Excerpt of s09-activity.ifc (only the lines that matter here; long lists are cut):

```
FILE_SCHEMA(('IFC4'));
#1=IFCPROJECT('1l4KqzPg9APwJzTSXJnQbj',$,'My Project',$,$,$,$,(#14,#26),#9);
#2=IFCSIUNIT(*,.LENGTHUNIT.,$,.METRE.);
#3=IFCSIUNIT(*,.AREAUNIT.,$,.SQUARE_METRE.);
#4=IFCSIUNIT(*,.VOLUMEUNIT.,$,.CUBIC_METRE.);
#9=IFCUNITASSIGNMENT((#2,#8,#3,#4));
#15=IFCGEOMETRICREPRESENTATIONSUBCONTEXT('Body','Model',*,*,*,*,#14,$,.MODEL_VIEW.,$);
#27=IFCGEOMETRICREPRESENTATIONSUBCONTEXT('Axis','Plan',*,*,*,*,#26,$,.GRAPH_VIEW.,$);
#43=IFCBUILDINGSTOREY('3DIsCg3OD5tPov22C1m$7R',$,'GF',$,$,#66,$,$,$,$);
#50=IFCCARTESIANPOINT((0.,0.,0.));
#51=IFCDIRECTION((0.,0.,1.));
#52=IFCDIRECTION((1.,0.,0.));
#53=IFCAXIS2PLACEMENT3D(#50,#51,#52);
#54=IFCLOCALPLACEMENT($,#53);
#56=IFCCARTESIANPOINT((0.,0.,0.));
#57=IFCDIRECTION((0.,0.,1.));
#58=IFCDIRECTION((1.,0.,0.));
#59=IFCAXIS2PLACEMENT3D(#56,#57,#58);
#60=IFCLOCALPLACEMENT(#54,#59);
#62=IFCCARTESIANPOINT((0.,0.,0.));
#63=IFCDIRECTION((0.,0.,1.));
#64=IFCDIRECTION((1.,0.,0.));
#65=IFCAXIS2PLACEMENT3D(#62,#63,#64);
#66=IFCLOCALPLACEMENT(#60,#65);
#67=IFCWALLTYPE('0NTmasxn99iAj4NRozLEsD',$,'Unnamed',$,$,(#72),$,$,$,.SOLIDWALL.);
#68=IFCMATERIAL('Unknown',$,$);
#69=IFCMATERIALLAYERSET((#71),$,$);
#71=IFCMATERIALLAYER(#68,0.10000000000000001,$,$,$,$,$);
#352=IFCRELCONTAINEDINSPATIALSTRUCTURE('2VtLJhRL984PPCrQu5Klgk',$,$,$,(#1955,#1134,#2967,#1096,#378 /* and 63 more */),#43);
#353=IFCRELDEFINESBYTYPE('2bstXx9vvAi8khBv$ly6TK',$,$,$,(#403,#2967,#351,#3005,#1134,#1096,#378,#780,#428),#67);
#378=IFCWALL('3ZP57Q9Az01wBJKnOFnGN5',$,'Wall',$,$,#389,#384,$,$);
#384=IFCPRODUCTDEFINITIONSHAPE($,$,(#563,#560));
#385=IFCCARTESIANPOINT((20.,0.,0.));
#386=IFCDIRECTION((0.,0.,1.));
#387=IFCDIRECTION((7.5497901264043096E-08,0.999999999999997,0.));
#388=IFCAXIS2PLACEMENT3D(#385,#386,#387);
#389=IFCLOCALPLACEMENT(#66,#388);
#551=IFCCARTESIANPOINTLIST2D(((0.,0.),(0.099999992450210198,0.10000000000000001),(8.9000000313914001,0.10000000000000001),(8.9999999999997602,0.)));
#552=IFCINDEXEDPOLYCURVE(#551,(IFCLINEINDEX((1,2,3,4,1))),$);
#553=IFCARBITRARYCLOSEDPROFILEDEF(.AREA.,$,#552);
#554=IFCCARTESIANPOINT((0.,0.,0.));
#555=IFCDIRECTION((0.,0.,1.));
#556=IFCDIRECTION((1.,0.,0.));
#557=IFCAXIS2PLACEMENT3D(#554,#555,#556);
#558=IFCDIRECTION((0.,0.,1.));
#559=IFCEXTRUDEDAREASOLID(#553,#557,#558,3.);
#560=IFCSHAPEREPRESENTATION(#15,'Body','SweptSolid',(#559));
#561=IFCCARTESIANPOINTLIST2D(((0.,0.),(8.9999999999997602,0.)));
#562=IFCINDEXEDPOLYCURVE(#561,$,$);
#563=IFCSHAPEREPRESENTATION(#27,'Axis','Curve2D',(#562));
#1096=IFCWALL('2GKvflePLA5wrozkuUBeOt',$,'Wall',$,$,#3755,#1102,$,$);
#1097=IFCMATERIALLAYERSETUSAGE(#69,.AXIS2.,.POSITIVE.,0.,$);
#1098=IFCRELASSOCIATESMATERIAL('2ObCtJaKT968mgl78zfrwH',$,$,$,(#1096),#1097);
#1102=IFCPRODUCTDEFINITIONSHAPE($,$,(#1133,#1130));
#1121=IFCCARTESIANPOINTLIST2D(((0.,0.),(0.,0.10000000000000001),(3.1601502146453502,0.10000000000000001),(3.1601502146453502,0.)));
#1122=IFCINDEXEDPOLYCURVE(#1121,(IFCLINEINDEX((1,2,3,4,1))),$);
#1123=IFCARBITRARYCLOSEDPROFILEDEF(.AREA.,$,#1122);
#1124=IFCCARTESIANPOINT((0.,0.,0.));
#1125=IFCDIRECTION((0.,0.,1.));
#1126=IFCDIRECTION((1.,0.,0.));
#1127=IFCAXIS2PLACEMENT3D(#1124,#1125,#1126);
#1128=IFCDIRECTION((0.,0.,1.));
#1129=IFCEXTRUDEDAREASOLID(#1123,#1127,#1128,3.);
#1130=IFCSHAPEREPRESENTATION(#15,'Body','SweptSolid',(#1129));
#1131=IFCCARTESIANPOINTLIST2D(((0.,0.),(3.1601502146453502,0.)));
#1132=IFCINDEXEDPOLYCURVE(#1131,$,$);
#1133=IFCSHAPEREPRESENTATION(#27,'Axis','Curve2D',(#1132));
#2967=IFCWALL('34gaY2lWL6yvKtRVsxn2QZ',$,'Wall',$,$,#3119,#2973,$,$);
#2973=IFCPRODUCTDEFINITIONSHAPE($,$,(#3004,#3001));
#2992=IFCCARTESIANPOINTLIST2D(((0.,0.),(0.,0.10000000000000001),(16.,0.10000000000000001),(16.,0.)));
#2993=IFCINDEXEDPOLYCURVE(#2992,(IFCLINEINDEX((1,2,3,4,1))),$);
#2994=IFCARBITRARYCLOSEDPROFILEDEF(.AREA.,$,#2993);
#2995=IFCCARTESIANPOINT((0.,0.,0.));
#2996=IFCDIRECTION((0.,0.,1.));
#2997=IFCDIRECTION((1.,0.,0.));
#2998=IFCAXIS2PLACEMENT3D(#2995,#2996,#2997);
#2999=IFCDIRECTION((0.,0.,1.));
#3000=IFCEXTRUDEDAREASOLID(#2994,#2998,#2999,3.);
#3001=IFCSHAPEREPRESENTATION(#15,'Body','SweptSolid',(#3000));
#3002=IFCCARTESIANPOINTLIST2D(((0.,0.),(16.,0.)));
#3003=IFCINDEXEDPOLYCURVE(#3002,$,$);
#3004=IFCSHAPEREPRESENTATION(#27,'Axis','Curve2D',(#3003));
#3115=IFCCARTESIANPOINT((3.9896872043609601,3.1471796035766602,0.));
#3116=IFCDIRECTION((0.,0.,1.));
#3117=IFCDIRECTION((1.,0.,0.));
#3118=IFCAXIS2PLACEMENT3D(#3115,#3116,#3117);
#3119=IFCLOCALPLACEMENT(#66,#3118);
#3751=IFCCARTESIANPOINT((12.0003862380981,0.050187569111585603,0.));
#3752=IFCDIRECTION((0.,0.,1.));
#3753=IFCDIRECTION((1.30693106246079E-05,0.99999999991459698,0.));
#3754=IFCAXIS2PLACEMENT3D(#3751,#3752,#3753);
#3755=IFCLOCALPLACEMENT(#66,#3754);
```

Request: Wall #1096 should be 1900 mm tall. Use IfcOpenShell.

```python
import ifcopenshell
import ifcopenshell.geom
import ifcopenshell.util.representation
import ifcopenshell.util.shape
import ifcopenshell.util.unit

model = ifcopenshell.open("s09-activity.ifc")
unit_scale = ifcopenshell.util.unit.calculate_unit_scale(model)
settings = ifcopenshell.geom.settings()


def volume(element):
    """Net volume in cubic metres, openings subtracted."""
    shape = ifcopenshell.geom.create_shape(settings, element)
    return ifcopenshell.util.shape.get_volume(shape.geometry)


wall = model.by_guid("2GKvflePLA5wrozkuUBeOt")
before = volume(wall)

body = ifcopenshell.util.representation.get_representation(wall, "Model", "Body")
solid = body.Items[0]
old_height = solid.Depth
solid.Depth = 1.9 / unit_scale
after = volume(wall)

print(f"height {old_height:g} -> {solid.Depth:g}, volume {before:.3f} -> {after:.3f} m3")

model.write("s09-activity_rev.ifc")
```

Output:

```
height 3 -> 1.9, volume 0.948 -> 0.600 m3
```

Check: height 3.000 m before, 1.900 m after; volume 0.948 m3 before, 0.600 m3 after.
